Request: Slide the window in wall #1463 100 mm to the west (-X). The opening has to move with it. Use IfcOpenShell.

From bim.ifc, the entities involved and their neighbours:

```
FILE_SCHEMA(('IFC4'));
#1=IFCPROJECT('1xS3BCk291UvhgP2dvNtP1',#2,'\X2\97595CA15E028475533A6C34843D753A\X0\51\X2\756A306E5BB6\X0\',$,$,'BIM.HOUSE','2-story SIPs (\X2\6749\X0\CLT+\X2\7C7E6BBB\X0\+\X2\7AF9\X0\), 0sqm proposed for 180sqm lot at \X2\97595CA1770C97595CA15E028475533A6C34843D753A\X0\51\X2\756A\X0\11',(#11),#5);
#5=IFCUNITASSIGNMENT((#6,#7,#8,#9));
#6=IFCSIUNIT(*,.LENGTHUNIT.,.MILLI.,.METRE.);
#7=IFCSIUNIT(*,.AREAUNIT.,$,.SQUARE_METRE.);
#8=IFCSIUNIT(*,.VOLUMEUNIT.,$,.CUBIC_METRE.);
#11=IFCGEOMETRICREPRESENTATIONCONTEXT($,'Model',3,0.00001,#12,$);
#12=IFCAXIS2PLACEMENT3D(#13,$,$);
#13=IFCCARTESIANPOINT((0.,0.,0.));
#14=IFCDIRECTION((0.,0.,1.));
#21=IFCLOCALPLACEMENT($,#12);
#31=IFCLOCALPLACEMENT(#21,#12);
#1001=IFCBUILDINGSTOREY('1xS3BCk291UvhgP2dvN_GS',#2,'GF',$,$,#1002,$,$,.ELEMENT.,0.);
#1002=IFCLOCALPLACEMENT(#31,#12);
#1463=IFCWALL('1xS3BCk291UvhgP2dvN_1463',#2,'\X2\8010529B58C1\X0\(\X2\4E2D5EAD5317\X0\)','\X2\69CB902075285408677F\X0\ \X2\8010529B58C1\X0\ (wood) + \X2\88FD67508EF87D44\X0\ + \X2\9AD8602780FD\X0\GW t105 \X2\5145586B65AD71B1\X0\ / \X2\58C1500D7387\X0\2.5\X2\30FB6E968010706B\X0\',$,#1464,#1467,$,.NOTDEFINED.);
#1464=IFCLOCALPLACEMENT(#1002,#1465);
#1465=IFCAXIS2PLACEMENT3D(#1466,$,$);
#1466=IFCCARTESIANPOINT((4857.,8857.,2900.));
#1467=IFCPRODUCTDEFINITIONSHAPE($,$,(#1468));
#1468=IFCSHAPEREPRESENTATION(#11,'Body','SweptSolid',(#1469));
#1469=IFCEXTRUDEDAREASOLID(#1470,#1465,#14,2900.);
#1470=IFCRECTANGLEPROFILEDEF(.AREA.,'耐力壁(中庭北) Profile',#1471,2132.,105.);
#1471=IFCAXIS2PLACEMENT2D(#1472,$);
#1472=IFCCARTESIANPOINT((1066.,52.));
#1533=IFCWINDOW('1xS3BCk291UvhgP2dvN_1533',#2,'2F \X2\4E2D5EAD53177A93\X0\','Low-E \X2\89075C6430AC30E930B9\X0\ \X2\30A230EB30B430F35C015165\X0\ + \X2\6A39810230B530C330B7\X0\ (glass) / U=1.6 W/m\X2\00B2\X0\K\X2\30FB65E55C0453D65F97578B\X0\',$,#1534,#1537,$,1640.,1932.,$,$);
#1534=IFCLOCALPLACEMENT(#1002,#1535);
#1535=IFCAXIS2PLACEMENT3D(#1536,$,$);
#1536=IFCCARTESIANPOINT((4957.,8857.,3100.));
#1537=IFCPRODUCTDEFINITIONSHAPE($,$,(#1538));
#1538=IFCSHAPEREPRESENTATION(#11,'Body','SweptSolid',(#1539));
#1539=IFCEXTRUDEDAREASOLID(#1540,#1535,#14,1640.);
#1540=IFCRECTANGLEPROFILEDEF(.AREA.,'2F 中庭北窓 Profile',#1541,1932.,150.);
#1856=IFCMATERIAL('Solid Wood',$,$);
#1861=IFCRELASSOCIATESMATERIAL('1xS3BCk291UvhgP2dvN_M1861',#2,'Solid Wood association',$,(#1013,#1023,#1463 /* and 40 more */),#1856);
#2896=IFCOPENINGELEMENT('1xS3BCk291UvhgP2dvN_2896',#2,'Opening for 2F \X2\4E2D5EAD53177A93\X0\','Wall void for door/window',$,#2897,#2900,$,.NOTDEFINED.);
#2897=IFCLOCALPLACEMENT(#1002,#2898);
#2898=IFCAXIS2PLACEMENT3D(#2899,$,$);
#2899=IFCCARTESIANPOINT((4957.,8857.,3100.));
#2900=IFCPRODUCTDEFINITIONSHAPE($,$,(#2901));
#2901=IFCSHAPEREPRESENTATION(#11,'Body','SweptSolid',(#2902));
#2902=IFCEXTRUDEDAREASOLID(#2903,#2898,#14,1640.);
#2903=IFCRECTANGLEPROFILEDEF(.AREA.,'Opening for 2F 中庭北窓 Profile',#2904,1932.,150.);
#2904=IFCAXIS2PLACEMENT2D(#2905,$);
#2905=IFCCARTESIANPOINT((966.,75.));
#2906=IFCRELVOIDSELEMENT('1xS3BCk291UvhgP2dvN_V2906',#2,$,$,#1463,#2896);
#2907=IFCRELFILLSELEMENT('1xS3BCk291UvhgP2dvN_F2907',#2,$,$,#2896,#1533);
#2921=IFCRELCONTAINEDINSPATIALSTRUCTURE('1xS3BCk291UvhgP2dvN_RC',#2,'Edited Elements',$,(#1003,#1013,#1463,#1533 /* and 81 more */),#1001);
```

```python
import ifcopenshell
import ifcopenshell.api.geometry
import ifcopenshell.util.placement

model = ifcopenshell.open("bim.ifc")

window = model.by_guid("1xS3BCk291UvhgP2dvN_1533")
opening = window.FillsVoids[0].RelatingOpeningElement
wall = opening.VoidsElements[0].RelatingBuildingElement

wall_matrix = ifcopenshell.util.placement.get_local_placement(wall.ObjectPlacement)
shift = wall_matrix[:3, 0] * -100.0
before = ifcopenshell.util.placement.get_local_placement(window.ObjectPlacement)[:3, 3].copy()

# The window is not placed relative to its opening, so move both.
for product in (opening, window):
    matrix = ifcopenshell.util.placement.get_local_placement(product.ObjectPlacement)
    matrix[:3, 3] += shift
    ifcopenshell.api.geometry.edit_object_placement(model, product=product, matrix=matrix, is_si=False)

after = ifcopenshell.util.placement.get_local_placement(window.ObjectPlacement)[:3, 3]
print("window moved by", (after - before).round(3) + 0.0)

model.write("bim-out.ifc")
```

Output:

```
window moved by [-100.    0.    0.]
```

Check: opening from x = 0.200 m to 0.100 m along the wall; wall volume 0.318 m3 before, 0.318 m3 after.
